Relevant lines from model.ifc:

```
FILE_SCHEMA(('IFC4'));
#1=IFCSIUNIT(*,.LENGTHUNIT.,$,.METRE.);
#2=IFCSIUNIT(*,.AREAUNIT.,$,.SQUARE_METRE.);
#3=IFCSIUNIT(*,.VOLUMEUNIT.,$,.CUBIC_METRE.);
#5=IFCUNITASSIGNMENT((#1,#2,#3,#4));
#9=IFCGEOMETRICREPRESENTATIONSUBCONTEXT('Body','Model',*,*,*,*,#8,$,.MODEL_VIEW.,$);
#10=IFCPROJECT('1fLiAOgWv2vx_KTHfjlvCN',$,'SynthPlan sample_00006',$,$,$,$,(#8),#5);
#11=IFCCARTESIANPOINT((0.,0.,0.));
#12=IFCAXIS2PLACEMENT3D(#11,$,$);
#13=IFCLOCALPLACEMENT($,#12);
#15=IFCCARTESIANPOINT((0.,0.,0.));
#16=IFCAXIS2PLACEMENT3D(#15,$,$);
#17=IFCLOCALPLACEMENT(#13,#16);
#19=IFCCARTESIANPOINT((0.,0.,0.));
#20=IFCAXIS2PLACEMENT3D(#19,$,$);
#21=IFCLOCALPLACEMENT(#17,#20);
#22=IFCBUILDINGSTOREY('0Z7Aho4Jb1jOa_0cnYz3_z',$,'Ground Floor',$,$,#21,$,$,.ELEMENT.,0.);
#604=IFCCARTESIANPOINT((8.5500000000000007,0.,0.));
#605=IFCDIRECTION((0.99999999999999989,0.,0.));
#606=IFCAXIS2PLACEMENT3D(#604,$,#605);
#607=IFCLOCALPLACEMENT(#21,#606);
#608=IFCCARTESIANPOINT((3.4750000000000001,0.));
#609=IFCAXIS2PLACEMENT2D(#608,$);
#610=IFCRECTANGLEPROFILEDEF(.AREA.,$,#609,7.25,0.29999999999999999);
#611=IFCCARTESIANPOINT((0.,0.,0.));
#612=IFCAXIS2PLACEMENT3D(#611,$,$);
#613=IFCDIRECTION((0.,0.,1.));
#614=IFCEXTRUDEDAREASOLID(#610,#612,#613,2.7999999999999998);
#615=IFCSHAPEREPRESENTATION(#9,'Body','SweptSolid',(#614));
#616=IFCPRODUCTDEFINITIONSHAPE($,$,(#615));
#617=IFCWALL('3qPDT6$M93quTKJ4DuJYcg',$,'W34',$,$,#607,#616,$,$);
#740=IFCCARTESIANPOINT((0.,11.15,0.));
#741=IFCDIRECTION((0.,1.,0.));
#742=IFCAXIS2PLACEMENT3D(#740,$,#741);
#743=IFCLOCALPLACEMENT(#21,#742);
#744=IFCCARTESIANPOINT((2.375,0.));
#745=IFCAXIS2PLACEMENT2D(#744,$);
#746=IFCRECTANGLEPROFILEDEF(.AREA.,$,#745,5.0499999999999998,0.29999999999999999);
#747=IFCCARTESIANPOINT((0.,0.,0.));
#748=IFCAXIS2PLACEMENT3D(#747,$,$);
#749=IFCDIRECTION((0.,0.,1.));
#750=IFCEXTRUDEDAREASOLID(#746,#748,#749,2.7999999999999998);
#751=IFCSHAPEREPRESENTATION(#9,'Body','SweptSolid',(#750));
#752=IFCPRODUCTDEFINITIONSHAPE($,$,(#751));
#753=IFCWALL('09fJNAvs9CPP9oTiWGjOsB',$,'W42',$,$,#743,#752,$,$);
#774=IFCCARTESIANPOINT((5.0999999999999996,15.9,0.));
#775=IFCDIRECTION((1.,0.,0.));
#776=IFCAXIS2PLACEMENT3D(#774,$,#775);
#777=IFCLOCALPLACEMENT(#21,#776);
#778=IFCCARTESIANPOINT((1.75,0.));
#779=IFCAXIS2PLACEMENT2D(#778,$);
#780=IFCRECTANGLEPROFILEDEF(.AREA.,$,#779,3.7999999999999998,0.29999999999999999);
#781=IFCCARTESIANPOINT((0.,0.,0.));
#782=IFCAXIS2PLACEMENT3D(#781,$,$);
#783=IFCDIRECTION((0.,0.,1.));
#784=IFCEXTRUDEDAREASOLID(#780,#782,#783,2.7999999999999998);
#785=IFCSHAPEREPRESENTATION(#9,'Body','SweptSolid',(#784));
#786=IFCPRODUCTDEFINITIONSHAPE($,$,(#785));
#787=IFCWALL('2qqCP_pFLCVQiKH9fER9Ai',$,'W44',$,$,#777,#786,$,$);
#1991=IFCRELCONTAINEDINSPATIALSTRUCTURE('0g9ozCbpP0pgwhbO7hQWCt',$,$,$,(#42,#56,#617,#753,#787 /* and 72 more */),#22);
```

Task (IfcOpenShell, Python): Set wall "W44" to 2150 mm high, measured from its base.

```python
import ifcopenshell
import ifcopenshell.geom
import ifcopenshell.util.representation
import ifcopenshell.util.shape
import ifcopenshell.util.unit

model = ifcopenshell.open("model.ifc")
unit_scale = ifcopenshell.util.unit.calculate_unit_scale(model)
settings = ifcopenshell.geom.settings()


def volume(element):
    """Net volume in cubic metres, openings subtracted."""
    shape = ifcopenshell.geom.create_shape(settings, element)
    return ifcopenshell.util.shape.get_volume(shape.geometry)


wall = model.by_id(787)
before = volume(wall)

body = ifcopenshell.util.representation.get_representation(wall, "Model", "Body")
solid = body.Items[0]
old_height = solid.Depth
solid.Depth = 2.15 / unit_scale
after = volume(wall)

print(f"height {old_height:g} -> {solid.Depth:g}, volume {before:.3f} -> {after:.3f} m3")

model.write("model_edited.ifc")
```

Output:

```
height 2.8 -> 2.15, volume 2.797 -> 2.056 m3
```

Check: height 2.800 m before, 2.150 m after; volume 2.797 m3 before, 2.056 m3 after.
